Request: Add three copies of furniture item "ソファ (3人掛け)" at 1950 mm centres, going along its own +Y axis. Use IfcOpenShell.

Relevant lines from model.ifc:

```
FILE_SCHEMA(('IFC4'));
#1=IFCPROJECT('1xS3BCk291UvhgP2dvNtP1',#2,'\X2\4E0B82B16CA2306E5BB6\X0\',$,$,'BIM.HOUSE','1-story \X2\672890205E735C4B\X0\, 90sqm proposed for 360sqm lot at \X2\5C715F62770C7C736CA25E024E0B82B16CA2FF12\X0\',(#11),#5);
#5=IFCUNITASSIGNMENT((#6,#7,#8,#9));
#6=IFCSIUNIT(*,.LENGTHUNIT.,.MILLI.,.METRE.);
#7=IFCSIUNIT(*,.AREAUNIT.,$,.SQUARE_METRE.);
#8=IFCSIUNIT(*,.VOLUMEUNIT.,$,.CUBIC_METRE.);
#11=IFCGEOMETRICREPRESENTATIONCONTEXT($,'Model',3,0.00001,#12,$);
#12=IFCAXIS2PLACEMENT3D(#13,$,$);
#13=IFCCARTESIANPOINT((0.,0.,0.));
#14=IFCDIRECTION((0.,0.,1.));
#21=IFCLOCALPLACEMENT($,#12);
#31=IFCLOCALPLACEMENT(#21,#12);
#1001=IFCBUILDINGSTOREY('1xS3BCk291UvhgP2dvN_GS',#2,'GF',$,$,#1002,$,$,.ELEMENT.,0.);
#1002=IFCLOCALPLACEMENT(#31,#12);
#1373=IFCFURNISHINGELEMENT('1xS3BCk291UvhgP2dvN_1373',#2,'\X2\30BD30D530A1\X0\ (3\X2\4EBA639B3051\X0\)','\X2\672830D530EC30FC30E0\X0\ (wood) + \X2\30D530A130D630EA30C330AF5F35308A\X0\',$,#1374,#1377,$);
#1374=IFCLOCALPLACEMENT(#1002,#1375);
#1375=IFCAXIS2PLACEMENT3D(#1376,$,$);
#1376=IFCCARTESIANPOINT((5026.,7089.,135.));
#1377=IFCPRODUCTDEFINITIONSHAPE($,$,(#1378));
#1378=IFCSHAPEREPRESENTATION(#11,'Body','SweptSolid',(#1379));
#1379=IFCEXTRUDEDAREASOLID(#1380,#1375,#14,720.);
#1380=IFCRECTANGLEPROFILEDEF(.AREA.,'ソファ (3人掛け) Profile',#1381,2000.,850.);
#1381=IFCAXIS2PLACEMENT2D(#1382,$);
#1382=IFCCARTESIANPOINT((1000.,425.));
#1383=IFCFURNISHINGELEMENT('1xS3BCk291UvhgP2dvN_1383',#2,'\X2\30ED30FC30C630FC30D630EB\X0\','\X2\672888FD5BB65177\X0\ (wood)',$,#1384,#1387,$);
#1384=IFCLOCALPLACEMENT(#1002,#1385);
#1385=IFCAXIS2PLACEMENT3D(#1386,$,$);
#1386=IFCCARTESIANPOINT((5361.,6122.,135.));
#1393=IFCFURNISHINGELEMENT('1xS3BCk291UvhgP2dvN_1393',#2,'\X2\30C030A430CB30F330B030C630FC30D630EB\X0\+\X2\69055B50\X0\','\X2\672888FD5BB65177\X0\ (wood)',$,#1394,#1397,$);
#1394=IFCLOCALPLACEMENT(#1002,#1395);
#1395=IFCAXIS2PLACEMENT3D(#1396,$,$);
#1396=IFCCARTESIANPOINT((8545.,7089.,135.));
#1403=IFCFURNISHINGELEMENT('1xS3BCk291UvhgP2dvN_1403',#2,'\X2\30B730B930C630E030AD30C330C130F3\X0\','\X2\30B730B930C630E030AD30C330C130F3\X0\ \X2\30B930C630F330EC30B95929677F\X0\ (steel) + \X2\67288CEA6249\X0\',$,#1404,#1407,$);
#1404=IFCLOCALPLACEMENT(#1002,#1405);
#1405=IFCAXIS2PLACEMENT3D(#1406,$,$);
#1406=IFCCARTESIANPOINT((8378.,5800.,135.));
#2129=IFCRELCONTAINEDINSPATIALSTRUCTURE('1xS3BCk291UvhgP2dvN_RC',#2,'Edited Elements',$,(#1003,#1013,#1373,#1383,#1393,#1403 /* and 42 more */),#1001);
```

```python
import ifcopenshell
import ifcopenshell.api.geometry
import ifcopenshell.api.root
import ifcopenshell.util.element
import ifcopenshell.util.placement
import ifcopenshell.util.unit

model = ifcopenshell.open("model.ifc")
unit_scale = ifcopenshell.util.unit.calculate_unit_scale(model)


def reuse_history(source, copy):
    """copy_class also copies each property set's owner history, people and application; keep the originals."""
    for rel in copy.IsDefinedBy:
        if rel.is_a("IfcRelDefinesByProperties") and (history := rel.RelatingPropertyDefinition.OwnerHistory):
            rel.RelatingPropertyDefinition.OwnerHistory = source.OwnerHistory
            ifcopenshell.util.element.remove_deep2(model, history)


source = model.by_guid("1xS3BCk291UvhgP2dvN_1373")
base = ifcopenshell.util.placement.get_local_placement(source.ObjectPlacement)
step = base[:3, 1] * 1.95 / unit_scale

for i in range(1, 4):
    copy = ifcopenshell.api.root.copy_class(model, product=source)
    copy.Representation = ifcopenshell.util.element.copy_deep(
        model, source.Representation, exclude=["IfcGeometricRepresentationContext", "IfcRepresentationMap"]
    )
    reuse_history(source, copy)
    matrix = base.copy()
    matrix[:3, 3] += i * step
    print("added at", matrix[:3, 3].round(3) + 0.0)
    ifcopenshell.api.geometry.edit_object_placement(model, product=copy, matrix=matrix, is_si=False)

model.write("model_rev.ifc")
```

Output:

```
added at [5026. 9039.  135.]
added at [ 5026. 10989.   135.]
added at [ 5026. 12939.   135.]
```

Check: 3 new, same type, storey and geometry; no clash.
